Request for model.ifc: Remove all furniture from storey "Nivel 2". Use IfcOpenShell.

First a look at what the model holds.

```python
import ifcopenshell
import ifcopenshell.util.element

model = ifcopenshell.open("model.ifc")
print(model.schema)
storey = next(s for s in model.by_type("IfcBuildingStorey") if s.Name == "Nivel 2")
furniture = [e for e in ifcopenshell.util.element.get_decomposition(storey) if e.is_a("IfcFurnishingElement")]
seen = {}
for e in furniture:
    element_type = ifcopenshell.util.element.get_type(e)
    name = element_type.Name if element_type not in (None, e) else None
    seen[name] = seen.get(name, 0) + 1
for name, count in sorted(seen.items(), key=str):
    print(count, "x", name)
```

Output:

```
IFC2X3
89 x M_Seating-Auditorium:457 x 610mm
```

```python
import ifcopenshell
import ifcopenshell.api.root
import ifcopenshell.util.element

model = ifcopenshell.open("model.ifc")

storey = next(s for s in model.by_type("IfcBuildingStorey") if s.Name == "Nivel 2")
furniture = [e for e in ifcopenshell.util.element.get_decomposition(storey) if e.is_a("IfcFurnishingElement")]

for e in furniture:
    ifcopenshell.api.root.remove_product(model, product=e)
print(len(furniture), "removed")

model.write("model_updated.ifc")
```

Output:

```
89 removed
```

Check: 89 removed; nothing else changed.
